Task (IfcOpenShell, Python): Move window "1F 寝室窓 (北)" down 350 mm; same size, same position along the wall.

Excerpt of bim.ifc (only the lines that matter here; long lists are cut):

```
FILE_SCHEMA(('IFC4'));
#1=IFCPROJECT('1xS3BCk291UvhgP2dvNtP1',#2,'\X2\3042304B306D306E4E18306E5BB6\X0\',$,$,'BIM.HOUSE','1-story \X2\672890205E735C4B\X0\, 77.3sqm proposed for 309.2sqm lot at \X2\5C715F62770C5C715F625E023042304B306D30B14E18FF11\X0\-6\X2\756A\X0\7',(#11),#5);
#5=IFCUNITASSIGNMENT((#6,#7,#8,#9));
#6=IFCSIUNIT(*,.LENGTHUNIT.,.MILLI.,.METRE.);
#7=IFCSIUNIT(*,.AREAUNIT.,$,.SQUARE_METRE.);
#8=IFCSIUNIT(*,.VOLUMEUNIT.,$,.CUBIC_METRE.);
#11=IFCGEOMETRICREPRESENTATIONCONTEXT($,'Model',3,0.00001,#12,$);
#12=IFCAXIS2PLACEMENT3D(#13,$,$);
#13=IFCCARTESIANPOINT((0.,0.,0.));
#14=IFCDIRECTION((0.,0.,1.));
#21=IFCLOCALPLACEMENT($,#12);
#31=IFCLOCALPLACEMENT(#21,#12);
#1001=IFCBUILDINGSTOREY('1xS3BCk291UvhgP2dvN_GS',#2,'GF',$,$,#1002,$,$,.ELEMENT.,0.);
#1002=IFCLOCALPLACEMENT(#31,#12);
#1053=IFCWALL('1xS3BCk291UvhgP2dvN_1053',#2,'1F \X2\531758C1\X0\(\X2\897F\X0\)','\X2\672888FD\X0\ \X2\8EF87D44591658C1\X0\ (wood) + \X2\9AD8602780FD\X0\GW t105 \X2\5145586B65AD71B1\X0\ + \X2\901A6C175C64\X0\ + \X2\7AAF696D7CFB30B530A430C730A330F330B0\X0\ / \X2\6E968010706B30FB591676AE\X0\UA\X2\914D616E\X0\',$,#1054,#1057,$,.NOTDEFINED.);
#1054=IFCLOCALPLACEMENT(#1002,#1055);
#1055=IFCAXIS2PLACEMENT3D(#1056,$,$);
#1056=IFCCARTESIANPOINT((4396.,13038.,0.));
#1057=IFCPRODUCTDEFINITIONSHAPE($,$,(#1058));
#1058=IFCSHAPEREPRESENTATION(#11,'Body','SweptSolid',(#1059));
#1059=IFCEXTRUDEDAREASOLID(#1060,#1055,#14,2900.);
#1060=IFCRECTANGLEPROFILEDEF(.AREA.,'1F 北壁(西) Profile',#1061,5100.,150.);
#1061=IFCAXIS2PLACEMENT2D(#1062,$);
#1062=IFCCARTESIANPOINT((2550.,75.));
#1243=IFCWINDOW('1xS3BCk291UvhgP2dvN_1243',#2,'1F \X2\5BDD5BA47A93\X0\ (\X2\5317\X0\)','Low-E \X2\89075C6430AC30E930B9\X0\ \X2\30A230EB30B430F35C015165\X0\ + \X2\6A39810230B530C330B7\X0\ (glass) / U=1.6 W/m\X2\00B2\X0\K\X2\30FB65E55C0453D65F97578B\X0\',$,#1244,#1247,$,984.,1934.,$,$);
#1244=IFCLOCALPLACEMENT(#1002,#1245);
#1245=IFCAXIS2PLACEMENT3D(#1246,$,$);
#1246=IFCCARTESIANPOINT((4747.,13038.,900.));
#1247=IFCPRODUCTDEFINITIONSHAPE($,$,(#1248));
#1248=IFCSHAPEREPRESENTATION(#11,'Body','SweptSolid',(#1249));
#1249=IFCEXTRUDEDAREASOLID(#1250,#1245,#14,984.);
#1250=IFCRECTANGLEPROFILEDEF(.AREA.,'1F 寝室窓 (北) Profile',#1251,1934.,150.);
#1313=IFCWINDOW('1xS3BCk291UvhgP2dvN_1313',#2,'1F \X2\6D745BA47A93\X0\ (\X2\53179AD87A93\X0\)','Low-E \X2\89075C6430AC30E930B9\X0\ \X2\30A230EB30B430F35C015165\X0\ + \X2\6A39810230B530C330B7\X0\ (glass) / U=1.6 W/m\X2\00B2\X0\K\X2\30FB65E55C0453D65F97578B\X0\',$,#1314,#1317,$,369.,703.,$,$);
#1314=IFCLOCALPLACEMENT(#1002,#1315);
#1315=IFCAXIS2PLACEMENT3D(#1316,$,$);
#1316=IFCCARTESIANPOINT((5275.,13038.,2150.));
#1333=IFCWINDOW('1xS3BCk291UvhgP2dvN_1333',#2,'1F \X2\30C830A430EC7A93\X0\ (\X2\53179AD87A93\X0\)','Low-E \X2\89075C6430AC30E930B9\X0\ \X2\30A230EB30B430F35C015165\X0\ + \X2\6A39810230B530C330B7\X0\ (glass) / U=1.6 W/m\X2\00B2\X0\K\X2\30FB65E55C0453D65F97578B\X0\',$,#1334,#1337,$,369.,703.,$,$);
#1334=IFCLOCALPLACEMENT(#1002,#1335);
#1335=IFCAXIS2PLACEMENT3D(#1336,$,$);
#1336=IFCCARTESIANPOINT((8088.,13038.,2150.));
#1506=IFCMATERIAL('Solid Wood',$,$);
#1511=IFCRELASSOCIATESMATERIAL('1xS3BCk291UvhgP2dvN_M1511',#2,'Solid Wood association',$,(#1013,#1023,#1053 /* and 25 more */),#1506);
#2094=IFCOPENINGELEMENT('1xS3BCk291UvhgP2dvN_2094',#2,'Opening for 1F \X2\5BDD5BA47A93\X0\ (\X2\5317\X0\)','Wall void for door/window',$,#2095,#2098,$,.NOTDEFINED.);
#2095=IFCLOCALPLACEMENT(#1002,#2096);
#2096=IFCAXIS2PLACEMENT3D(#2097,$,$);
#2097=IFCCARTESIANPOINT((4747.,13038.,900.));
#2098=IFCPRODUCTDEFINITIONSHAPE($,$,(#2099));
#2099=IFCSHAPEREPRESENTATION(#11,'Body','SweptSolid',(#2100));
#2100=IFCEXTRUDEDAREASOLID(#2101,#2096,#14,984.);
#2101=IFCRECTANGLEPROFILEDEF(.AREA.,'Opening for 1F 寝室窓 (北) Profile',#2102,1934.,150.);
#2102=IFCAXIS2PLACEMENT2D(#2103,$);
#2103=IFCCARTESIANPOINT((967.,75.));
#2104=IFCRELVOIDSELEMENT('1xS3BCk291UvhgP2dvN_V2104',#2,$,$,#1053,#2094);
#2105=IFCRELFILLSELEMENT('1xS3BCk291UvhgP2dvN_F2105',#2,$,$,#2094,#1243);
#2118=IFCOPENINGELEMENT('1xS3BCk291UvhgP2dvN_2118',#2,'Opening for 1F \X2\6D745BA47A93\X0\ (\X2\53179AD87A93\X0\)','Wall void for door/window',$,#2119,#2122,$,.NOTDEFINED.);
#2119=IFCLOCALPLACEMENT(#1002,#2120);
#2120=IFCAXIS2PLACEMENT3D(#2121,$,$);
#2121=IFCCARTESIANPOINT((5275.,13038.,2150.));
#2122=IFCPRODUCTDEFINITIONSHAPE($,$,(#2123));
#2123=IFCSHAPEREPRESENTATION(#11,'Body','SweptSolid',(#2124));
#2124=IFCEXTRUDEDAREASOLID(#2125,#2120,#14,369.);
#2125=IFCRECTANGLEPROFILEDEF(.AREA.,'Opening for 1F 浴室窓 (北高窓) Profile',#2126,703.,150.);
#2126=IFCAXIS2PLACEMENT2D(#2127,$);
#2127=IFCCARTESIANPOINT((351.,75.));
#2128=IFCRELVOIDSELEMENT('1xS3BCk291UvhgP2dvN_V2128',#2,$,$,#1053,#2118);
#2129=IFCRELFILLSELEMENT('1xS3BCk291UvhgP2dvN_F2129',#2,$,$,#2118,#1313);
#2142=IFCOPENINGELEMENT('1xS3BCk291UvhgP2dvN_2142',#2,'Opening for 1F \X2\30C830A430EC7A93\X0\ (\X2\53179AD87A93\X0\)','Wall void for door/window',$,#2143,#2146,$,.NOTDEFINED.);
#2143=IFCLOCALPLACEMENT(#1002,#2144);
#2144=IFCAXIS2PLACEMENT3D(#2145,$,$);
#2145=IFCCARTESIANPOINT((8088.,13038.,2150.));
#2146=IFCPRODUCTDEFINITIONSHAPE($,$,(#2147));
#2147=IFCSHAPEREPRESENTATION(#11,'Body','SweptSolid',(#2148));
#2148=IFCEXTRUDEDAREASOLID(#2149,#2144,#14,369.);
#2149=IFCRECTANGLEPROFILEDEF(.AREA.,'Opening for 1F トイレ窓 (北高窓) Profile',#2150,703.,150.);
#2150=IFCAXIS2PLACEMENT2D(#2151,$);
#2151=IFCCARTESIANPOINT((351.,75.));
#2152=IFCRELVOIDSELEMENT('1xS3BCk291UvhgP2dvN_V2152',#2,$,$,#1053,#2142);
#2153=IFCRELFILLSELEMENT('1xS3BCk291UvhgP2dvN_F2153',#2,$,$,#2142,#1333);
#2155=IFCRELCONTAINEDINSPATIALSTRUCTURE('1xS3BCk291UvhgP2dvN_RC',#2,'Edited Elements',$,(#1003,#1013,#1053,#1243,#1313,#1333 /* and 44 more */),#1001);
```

```python
import numpy as np
import ifcopenshell
import ifcopenshell.api.geometry
import ifcopenshell.util.placement
import ifcopenshell.util.unit

model = ifcopenshell.open("bim.ifc")
unit_scale = ifcopenshell.util.unit.calculate_unit_scale(model)

window = model.by_id(1243)
opening = window.FillsVoids[0].RelatingOpeningElement
dz = -0.35 / unit_scale

shift = np.array([0.0, 0.0, dz])
# The window is not placed relative to its opening, so move both.
for product in (opening, window):
    matrix = ifcopenshell.util.placement.get_local_placement(product.ObjectPlacement)
    matrix[:3, 3] += shift
    ifcopenshell.api.geometry.edit_object_placement(model, product=product, matrix=matrix, is_si=False)

print(f"moved by {dz * unit_scale:+.3f} m")

model.write("bim_rev.ifc")
```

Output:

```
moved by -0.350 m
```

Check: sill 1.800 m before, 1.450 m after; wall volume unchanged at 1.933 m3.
